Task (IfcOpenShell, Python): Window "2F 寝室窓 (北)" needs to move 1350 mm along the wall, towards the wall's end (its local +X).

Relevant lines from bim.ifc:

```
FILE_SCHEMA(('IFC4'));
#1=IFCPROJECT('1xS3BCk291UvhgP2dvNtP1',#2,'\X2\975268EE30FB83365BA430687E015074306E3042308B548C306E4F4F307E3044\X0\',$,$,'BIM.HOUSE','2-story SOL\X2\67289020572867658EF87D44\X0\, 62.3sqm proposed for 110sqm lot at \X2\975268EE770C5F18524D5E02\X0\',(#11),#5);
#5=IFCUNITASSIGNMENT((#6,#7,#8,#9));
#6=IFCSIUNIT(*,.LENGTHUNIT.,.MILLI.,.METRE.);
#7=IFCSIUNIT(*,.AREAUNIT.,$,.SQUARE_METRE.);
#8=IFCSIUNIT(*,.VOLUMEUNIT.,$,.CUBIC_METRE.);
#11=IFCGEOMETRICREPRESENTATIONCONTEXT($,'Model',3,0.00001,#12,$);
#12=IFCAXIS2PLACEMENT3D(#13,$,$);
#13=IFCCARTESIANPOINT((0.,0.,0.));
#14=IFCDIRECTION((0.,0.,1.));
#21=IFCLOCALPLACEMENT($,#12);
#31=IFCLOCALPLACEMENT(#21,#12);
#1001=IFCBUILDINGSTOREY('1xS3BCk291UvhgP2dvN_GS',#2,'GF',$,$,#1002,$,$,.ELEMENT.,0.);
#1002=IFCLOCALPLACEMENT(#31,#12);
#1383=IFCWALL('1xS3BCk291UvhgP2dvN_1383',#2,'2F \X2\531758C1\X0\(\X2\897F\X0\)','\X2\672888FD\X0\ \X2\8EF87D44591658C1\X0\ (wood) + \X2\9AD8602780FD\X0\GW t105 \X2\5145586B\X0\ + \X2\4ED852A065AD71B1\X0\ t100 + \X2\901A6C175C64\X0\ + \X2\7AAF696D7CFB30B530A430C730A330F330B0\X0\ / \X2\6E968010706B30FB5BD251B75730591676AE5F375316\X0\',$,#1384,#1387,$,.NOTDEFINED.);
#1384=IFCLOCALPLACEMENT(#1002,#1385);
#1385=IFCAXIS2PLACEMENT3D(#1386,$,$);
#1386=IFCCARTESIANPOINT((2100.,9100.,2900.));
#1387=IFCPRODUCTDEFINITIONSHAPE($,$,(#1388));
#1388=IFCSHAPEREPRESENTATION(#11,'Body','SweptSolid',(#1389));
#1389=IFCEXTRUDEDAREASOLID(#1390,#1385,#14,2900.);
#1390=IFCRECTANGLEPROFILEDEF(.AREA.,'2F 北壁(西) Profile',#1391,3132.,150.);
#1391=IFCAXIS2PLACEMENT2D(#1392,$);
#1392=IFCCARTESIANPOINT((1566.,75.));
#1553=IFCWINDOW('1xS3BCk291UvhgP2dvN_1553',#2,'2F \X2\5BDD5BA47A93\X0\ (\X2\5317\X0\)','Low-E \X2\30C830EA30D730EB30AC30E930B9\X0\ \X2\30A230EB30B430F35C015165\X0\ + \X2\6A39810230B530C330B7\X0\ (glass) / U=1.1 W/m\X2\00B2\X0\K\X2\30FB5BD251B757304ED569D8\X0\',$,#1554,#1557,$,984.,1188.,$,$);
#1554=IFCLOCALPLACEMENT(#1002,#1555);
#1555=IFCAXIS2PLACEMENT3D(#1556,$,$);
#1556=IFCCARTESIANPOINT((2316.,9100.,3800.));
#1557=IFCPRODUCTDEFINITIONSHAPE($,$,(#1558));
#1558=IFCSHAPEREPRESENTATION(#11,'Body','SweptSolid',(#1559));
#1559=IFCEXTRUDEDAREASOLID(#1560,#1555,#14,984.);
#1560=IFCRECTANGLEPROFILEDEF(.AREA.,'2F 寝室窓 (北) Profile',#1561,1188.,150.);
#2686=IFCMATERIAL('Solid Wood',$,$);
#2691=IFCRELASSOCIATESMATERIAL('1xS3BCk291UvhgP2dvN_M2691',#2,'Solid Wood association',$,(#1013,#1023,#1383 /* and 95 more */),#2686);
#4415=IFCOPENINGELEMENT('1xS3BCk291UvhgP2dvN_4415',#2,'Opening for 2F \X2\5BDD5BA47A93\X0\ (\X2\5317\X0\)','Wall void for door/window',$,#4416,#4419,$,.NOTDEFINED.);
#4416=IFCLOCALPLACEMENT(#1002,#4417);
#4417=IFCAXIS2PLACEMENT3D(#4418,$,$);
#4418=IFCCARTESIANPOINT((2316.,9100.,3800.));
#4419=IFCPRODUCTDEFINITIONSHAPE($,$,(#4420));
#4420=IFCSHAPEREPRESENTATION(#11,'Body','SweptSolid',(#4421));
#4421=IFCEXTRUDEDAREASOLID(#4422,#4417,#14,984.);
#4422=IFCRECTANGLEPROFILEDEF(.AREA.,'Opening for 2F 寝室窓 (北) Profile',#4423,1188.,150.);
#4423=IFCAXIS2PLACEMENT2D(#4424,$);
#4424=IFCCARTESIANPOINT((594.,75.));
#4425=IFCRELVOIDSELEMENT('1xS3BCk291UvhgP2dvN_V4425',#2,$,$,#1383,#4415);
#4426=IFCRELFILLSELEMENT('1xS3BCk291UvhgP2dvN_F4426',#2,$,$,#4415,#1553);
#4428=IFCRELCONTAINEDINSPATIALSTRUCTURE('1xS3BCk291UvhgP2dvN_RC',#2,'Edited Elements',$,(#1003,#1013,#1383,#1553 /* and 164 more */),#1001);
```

```python
import ifcopenshell
import ifcopenshell.api.geometry
import ifcopenshell.util.placement
import ifcopenshell.util.unit

model = ifcopenshell.open("bim.ifc")
unit_scale = ifcopenshell.util.unit.calculate_unit_scale(model)

window = model.by_guid("1xS3BCk291UvhgP2dvN_1553")
opening = window.FillsVoids[0].RelatingOpeningElement
wall = opening.VoidsElements[0].RelatingBuildingElement

wall_matrix = ifcopenshell.util.placement.get_local_placement(wall.ObjectPlacement)
shift = wall_matrix[:3, 0] * 1.35 / unit_scale
before = ifcopenshell.util.placement.get_local_placement(window.ObjectPlacement)[:3, 3].copy()

# The window is not placed relative to its opening, so move both.
for product in (opening, window):
    matrix = ifcopenshell.util.placement.get_local_placement(product.ObjectPlacement)
    matrix[:3, 3] += shift
    ifcopenshell.api.geometry.edit_object_placement(model, product=product, matrix=matrix, is_si=False)

after = ifcopenshell.util.placement.get_local_placement(window.ObjectPlacement)[:3, 3]
print("window moved by", (after - before).round(3) + 0.0)

model.write("bim_v2.ifc")
```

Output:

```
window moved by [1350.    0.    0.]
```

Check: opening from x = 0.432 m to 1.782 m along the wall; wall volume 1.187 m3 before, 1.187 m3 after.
